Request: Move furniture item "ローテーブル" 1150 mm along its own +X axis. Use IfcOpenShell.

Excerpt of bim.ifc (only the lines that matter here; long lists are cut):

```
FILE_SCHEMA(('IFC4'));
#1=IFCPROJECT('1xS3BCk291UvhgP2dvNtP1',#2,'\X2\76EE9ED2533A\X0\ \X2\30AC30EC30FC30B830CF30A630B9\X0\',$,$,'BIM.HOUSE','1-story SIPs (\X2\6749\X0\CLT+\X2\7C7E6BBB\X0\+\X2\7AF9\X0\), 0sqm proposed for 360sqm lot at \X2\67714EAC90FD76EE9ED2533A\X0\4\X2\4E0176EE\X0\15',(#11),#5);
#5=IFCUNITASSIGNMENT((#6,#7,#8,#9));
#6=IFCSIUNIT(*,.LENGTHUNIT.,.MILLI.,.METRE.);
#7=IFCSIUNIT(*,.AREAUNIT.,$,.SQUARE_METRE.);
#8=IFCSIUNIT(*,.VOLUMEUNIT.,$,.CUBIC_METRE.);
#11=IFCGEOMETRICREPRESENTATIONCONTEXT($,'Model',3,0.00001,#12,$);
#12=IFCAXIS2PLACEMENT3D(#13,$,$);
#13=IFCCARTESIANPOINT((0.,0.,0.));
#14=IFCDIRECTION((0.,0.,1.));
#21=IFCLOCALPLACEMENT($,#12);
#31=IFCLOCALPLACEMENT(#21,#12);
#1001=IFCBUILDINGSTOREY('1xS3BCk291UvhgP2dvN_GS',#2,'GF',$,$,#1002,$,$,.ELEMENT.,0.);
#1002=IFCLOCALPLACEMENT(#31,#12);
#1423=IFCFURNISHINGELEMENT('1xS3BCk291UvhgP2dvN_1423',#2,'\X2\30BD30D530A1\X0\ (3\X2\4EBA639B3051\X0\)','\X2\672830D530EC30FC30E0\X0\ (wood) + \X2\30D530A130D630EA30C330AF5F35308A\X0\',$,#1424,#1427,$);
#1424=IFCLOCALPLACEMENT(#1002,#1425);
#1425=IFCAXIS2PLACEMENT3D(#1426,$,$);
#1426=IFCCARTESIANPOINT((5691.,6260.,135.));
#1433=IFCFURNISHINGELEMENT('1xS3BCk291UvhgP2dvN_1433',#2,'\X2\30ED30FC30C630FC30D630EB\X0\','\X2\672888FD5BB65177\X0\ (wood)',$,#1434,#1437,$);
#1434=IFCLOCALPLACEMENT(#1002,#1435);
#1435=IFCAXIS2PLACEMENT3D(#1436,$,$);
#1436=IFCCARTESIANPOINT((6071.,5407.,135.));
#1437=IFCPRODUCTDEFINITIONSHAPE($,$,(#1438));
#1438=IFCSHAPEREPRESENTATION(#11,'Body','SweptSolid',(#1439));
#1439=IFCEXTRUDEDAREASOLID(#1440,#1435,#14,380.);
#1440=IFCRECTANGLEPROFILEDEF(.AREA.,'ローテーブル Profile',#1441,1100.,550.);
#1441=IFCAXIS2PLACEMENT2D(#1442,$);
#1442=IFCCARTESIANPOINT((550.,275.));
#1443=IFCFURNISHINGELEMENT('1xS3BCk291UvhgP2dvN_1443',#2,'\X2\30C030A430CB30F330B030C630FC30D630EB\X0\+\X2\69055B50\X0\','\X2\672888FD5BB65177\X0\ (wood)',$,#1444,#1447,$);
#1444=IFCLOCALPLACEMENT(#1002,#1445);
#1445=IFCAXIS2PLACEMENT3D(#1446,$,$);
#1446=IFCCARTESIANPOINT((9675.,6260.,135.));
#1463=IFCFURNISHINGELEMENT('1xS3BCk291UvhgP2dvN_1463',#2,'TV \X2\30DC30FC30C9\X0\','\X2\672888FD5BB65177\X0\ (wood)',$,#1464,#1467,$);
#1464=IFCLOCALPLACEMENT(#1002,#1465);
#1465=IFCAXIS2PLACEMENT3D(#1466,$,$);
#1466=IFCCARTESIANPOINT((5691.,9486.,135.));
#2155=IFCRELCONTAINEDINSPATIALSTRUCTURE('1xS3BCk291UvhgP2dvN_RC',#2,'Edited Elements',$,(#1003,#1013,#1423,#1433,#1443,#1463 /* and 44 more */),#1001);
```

```python
import ifcopenshell
import ifcopenshell.api.geometry
import ifcopenshell.util.placement

model = ifcopenshell.open("bim.ifc")

item = model.by_guid("1xS3BCk291UvhgP2dvN_1433")
matrix = ifcopenshell.util.placement.get_local_placement(item.ObjectPlacement)
matrix[:3, 3] += matrix[:3, 0] * 1150.0
ifcopenshell.api.geometry.edit_object_placement(model, product=item, matrix=matrix, is_si=False)

print(ifcopenshell.util.placement.get_local_placement(item.ObjectPlacement).round(3) + 0.0)

model.write("bim_rev.ifc")
```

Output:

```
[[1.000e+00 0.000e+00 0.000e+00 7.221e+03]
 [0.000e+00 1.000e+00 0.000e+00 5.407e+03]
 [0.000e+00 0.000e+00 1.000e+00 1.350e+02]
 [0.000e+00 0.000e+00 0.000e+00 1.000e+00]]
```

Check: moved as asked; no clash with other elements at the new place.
